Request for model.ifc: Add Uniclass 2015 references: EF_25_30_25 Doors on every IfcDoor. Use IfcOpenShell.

First a look at what the model holds.

```python
import ifcopenshell

model = ifcopenshell.open("model.ifc")
print(model.schema)
print("classifications:", [c.Name for c in model.by_type("IfcClassification")])
for ifc_class in ("IfcDoor", "IfcRoof", "IfcStair", "IfcWall", "IfcWindow"):
    print(ifc_class, len(model.by_type(ifc_class)))
```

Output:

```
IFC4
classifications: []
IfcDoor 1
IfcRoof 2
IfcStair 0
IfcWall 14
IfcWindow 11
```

```python
import ifcopenshell
import ifcopenshell.api.classification

model = ifcopenshell.open("model.ifc")

system = ifcopenshell.api.classification.add_classification(model, classification="Uniclass 2015")

codes = {
    "IfcDoor": ("EF_25_30_25", "Doors"),
}
for ifc_class, (code, name) in codes.items():
    products = model.by_type(ifc_class)
    ifcopenshell.api.classification.add_reference(
        model, products=products, classification=system, identification=code, name=name
    )
    print(code, len(products))

model.write("model_updated.ifc")
```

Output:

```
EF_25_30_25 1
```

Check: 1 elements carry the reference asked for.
